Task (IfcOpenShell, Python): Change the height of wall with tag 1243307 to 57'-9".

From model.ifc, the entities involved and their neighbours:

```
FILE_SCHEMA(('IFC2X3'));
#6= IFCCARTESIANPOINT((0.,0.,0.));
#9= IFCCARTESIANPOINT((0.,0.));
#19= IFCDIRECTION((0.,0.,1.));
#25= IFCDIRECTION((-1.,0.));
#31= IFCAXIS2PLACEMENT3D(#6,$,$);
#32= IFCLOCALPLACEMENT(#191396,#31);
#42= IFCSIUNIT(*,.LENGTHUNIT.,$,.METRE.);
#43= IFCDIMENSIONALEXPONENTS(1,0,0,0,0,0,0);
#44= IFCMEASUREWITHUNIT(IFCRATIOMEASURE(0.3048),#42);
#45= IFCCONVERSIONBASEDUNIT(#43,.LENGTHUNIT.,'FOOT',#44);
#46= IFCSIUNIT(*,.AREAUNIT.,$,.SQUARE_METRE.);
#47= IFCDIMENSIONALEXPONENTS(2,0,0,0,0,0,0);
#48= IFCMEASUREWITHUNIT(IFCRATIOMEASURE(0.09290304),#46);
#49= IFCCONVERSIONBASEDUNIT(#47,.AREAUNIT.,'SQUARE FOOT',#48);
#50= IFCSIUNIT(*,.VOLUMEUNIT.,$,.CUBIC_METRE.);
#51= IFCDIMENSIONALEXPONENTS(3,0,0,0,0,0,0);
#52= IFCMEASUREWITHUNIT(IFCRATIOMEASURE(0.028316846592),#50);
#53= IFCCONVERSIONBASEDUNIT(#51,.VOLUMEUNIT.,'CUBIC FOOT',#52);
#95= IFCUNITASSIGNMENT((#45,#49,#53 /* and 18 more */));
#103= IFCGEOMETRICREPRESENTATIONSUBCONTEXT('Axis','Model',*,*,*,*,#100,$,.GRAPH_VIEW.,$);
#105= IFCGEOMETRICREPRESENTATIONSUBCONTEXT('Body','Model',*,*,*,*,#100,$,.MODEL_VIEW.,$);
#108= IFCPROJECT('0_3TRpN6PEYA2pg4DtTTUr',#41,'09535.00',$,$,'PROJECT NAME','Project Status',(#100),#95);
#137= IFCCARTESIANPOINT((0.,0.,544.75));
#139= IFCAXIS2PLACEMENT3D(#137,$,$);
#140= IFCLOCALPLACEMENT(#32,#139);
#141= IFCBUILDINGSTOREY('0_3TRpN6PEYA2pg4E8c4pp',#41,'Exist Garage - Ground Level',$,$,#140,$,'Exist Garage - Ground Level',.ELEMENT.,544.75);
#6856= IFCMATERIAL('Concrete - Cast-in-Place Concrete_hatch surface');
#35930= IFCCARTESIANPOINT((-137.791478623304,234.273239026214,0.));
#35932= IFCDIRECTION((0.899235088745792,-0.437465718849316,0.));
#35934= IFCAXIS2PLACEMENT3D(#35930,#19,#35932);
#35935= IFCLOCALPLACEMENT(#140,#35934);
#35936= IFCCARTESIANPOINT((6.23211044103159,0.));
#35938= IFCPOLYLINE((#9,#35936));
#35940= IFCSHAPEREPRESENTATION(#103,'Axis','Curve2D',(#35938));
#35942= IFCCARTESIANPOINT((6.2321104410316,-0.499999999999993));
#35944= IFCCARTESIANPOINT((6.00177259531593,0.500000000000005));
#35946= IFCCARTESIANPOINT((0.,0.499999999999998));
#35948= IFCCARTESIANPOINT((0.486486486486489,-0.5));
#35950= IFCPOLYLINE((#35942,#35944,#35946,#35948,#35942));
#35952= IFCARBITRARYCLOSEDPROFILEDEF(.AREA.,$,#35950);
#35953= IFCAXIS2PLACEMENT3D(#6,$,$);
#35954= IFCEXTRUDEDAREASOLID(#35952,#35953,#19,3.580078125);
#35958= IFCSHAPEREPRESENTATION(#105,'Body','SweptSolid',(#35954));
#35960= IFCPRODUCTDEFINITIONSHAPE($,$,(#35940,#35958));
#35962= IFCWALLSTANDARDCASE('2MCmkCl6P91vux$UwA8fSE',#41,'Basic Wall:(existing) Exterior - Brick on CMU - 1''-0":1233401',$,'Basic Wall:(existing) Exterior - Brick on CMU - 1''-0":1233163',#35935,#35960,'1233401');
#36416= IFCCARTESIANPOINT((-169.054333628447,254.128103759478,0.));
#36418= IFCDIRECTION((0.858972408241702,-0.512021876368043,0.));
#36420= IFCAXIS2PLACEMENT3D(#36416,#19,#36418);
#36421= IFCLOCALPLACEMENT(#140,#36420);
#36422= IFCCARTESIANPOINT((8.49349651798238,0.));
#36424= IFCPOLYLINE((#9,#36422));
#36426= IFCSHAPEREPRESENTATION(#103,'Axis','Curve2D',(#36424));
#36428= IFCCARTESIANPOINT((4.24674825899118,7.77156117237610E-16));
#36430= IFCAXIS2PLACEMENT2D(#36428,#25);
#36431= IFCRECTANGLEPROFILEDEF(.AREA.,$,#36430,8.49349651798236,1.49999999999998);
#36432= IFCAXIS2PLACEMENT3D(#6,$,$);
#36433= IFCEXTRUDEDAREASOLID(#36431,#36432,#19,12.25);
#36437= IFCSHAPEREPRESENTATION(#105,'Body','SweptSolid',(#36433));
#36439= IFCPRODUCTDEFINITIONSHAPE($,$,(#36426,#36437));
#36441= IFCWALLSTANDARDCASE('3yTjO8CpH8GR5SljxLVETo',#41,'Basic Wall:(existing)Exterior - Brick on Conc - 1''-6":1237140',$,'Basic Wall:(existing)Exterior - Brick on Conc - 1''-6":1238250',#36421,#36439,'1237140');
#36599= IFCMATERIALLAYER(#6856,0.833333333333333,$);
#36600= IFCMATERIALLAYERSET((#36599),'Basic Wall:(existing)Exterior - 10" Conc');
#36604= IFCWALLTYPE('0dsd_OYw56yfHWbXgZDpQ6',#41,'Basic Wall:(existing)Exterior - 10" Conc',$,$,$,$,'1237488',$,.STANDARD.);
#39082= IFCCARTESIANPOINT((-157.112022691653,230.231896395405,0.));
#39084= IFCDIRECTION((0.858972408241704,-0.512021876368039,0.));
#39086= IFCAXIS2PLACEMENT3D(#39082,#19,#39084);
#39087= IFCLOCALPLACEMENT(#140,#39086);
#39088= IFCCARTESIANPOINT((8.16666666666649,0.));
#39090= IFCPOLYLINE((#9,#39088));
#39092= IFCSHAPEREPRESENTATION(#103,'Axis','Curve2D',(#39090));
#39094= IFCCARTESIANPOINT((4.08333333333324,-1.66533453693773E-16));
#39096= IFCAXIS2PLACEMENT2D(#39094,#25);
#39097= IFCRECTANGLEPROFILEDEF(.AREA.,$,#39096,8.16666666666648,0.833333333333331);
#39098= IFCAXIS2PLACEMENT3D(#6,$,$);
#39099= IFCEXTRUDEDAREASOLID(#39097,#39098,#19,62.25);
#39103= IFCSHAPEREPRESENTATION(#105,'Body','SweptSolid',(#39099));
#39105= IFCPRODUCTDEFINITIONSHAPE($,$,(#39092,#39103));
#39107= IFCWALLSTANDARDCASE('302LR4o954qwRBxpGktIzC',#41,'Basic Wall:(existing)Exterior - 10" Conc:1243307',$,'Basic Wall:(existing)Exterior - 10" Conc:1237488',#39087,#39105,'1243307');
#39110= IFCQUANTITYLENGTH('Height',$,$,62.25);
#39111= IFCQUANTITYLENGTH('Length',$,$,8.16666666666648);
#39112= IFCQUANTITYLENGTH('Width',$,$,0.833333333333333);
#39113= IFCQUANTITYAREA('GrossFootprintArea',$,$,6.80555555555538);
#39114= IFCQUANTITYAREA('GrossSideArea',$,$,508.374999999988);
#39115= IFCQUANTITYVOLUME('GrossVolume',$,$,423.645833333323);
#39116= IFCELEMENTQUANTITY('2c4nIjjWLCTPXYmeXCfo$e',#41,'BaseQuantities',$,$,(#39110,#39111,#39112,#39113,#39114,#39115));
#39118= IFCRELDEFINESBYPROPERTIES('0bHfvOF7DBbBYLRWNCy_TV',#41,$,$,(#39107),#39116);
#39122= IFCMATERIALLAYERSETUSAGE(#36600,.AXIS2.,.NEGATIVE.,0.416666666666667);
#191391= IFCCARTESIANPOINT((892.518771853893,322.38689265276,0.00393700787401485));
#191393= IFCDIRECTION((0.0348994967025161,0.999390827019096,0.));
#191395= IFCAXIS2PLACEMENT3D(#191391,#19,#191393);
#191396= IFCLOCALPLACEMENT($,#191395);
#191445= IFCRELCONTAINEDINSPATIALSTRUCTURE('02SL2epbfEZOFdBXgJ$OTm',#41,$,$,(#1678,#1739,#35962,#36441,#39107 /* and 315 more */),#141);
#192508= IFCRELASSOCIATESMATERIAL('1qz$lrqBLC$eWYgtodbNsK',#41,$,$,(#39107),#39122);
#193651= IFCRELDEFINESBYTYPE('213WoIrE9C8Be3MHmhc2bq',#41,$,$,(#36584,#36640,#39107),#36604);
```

```python
import ifcopenshell
import ifcopenshell.api.pset
import ifcopenshell.geom
import ifcopenshell.util.element
import ifcopenshell.util.representation
import ifcopenshell.util.shape
import ifcopenshell.util.unit

model = ifcopenshell.open("model.ifc")
unit_scale = ifcopenshell.util.unit.calculate_unit_scale(model)
area_scale = ifcopenshell.util.unit.calculate_unit_scale(model, "AREAUNIT")
volume_scale = ifcopenshell.util.unit.calculate_unit_scale(model, "VOLUMEUNIT")
settings = ifcopenshell.geom.settings()


def volume(element):
    """Net volume in cubic metres, openings subtracted."""
    shape = ifcopenshell.geom.create_shape(settings, element)
    return ifcopenshell.util.shape.get_volume(shape.geometry)


wall = model.by_id(39107)
before = volume(wall)

body = ifcopenshell.util.representation.get_representation(wall, "Model", "Body")
solid = body.Items[0]
old_height = solid.Depth
solid.Depth = 693 * 0.0254 / unit_scale
after = volume(wall)

# Update the stored height, areas and volumes.
qto = model.by_id(ifcopenshell.util.element.get_pset(wall, "BaseQuantities", should_inherit=False)["id"])
ifcopenshell.api.pset.edit_qto(model, qto=qto, properties={
    "Height": solid.Depth,
    "GrossSideArea": ifcopenshell.util.element.get_pset(wall, "BaseQuantities", "GrossSideArea") * solid.Depth / old_height,
    "GrossVolume": ifcopenshell.util.element.get_pset(wall, "BaseQuantities", "GrossVolume") * solid.Depth / old_height,
})

print(f"height {old_height:g} -> {solid.Depth:g}, volume {before:.3f} -> {after:.3f} m3")

model.write("model_edited.ifc")
```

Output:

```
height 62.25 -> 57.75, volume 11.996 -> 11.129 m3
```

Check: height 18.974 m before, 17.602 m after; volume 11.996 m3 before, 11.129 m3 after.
